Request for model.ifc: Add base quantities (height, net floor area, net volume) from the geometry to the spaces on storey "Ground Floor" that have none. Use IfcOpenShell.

First a look at what the model holds.

```python
import ifcopenshell
import ifcopenshell.util.element
import ifcopenshell.util.unit

model = ifcopenshell.open("model.ifc")
print(model.schema)
for unit_type in ("LENGTHUNIT", "AREAUNIT", "VOLUMEUNIT"):
    print(unit_type, ifcopenshell.util.unit.calculate_unit_scale(model, unit_type))
storey = next(s for s in model.by_type("IfcBuildingStorey") if s.Name == "Ground Floor")
spaces = [e for e in ifcopenshell.util.element.get_decomposition(storey) if e.is_a("IfcSpace")]
for e in sorted(spaces, key=lambda e: e.id()):
    print(e.id(), e.is_a(), e.Name, list(ifcopenshell.util.element.get_psets(e, qtos_only=True)), sep=" | ")
```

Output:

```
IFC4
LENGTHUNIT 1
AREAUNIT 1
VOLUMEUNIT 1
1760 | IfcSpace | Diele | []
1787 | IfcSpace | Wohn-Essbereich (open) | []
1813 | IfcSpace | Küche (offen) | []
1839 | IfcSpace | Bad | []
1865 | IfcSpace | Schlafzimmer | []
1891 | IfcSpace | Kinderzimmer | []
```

```python
import ifcopenshell
import ifcopenshell.api.pset
import ifcopenshell.geom
import ifcopenshell.util.element
import ifcopenshell.util.shape
import ifcopenshell.util.unit

model = ifcopenshell.open("model.ifc")
unit_scale = ifcopenshell.util.unit.calculate_unit_scale(model)
area_scale = ifcopenshell.util.unit.calculate_unit_scale(model, "AREAUNIT")
volume_scale = ifcopenshell.util.unit.calculate_unit_scale(model, "VOLUMEUNIT")
settings = ifcopenshell.geom.settings()

storey = next(s for s in model.by_type("IfcBuildingStorey") if s.Name == "Ground Floor")
spaces = [e for e in ifcopenshell.util.element.get_decomposition(storey) if e.is_a("IfcSpace")]

for e in sorted(spaces, key=lambda e: e.id()):
    if ifcopenshell.util.element.get_psets(e, qtos_only=True, should_inherit=False):
        continue
    # Geometry comes back in metres, in the element's own axes.
    shape = ifcopenshell.geom.create_shape(settings, e)
    values = {
        "Height": ifcopenshell.util.shape.get_z(shape.geometry) / unit_scale,
        "NetFloorArea": ifcopenshell.util.shape.get_footprint_area(shape.geometry) / area_scale,
        "NetVolume": ifcopenshell.util.shape.get_volume(shape.geometry) / volume_scale,
    }
    qto = ifcopenshell.api.pset.add_qto(model, product=e, name="Qto_SpaceBaseQuantities")
    ifcopenshell.api.pset.edit_qto(model, qto=qto, properties=values)
    print(e.id(), {k: round(v, 3) for k, v in values.items()})

model.write("model-out.ifc")
```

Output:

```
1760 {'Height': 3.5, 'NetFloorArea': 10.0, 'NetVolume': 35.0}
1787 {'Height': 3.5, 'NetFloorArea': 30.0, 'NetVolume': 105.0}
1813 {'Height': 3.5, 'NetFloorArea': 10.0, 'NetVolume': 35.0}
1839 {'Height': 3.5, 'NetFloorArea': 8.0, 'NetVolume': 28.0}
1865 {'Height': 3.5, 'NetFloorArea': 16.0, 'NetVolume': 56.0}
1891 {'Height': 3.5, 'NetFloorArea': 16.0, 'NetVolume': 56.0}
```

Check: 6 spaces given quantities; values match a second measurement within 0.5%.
